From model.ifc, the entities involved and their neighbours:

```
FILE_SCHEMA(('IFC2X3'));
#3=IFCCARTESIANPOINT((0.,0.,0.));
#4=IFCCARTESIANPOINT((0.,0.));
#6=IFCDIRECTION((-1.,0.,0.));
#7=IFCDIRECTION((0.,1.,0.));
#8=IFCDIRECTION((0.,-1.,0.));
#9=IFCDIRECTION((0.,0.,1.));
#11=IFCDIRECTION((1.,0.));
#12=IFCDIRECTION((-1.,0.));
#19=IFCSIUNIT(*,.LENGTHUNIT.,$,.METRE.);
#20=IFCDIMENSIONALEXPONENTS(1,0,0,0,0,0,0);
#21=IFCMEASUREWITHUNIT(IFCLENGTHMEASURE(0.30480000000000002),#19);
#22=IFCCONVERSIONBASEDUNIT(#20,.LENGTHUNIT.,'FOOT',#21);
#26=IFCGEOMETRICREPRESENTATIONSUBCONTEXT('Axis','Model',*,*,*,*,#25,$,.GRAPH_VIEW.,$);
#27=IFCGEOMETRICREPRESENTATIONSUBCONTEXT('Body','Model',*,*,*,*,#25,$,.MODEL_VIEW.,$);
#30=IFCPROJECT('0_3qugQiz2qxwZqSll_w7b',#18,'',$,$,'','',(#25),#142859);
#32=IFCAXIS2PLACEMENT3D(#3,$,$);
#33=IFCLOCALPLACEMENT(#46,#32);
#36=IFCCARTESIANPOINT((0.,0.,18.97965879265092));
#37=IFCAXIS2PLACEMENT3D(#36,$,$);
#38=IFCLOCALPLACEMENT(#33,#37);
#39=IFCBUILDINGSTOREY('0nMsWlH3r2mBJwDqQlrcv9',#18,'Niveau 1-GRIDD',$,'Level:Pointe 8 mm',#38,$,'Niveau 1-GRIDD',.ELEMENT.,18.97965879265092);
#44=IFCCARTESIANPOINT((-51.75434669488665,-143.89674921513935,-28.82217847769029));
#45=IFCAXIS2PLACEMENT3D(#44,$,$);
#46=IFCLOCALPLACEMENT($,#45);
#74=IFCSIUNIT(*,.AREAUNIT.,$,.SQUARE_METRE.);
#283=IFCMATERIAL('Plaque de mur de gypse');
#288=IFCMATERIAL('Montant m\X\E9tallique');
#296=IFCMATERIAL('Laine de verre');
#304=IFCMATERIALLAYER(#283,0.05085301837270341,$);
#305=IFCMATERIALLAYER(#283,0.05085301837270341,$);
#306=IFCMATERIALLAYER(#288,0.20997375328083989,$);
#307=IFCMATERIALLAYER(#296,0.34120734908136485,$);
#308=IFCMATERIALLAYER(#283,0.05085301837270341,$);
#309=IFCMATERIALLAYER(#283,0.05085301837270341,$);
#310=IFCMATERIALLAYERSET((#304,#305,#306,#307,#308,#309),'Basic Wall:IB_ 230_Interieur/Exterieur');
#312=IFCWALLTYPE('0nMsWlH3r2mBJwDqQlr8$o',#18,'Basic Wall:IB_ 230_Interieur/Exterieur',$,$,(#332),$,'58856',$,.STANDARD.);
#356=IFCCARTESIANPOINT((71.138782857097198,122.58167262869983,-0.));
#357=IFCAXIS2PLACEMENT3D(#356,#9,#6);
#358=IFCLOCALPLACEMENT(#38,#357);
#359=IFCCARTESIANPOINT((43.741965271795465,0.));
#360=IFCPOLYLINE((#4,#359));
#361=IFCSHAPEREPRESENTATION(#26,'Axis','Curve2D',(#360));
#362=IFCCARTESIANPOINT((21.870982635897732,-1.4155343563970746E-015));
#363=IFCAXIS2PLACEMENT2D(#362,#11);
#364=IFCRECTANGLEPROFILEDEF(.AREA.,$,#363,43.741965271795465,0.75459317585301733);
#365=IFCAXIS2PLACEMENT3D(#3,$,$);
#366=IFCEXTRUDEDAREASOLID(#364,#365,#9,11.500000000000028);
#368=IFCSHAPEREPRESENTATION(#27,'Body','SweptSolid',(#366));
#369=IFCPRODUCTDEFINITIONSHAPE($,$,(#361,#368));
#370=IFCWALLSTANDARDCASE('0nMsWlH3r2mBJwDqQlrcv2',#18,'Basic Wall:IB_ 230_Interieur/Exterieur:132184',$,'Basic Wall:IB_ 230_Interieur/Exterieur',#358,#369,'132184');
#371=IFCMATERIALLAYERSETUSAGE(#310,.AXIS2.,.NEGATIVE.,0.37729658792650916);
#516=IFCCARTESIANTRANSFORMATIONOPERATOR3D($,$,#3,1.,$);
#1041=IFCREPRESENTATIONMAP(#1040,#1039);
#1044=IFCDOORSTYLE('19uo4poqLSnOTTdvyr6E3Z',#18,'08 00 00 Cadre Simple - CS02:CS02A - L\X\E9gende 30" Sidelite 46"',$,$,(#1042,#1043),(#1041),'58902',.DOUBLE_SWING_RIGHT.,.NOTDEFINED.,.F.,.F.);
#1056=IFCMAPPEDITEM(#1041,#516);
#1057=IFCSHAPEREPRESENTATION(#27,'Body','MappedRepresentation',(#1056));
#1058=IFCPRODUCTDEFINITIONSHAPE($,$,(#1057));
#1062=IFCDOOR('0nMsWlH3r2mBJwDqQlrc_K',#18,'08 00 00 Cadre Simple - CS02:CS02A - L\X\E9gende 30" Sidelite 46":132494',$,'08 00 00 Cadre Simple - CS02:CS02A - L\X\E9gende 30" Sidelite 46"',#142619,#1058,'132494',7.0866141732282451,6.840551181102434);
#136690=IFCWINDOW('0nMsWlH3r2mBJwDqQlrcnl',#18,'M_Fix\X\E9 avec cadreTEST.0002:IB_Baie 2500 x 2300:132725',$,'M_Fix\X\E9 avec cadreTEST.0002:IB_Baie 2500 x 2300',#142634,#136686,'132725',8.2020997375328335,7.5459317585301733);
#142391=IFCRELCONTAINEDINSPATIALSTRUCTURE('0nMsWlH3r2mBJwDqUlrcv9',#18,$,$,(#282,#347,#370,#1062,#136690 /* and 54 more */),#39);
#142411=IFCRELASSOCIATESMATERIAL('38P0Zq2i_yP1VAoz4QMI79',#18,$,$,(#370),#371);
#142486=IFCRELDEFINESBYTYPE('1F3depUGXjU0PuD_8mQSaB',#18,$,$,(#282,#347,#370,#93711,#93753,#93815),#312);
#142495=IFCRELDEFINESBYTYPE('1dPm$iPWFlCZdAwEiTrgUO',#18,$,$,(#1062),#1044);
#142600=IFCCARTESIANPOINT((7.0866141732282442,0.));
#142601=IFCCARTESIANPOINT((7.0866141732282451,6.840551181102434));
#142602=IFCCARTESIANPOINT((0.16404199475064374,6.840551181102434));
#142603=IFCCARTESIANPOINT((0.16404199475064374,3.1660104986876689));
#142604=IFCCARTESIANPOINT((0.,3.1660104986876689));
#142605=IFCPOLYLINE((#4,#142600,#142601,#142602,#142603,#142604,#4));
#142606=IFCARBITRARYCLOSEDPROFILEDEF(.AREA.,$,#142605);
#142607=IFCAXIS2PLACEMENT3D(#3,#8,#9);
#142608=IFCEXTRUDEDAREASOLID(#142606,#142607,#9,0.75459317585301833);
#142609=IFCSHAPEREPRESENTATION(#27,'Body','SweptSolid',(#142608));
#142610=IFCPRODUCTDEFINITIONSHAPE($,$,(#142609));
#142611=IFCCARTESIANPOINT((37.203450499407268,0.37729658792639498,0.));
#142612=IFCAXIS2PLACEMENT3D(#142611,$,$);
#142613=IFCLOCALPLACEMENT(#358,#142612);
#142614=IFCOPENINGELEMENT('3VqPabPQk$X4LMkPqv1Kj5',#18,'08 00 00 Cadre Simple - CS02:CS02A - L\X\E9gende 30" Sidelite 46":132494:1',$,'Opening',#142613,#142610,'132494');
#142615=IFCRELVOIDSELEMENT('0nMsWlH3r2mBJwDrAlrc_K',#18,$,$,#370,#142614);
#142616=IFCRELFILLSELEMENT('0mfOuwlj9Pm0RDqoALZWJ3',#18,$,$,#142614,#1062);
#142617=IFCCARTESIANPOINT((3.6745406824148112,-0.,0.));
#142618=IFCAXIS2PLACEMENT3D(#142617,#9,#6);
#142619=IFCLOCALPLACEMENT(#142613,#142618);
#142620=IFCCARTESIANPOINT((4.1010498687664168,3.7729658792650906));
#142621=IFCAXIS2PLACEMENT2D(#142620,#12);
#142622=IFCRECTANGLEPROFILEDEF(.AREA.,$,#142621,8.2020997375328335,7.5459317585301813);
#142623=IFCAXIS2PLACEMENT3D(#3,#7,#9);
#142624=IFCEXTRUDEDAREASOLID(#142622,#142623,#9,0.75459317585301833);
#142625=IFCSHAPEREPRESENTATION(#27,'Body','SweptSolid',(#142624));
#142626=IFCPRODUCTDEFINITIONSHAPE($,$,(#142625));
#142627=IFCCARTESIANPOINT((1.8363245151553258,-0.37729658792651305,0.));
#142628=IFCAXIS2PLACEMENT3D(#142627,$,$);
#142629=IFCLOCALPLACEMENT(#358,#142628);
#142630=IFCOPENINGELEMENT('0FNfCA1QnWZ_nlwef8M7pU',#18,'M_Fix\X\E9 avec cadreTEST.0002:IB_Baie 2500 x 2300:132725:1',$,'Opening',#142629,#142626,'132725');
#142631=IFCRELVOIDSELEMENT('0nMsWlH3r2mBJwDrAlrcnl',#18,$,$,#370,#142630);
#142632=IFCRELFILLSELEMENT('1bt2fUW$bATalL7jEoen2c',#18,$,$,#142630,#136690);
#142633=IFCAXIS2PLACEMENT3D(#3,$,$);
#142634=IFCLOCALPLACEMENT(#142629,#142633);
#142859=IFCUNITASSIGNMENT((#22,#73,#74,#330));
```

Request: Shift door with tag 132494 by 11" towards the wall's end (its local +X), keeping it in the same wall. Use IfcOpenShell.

```python
import ifcopenshell
import ifcopenshell.api.geometry
import ifcopenshell.util.placement
import ifcopenshell.util.unit

model = ifcopenshell.open("model.ifc")
unit_scale = ifcopenshell.util.unit.calculate_unit_scale(model)

door = model.by_guid("0nMsWlH3r2mBJwDqQlrc_K")
opening = door.FillsVoids[0].RelatingOpeningElement
wall = opening.VoidsElements[0].RelatingBuildingElement

wall_matrix = ifcopenshell.util.placement.get_local_placement(wall.ObjectPlacement)
shift = wall_matrix[:3, 0] * 11 * 0.0254 / unit_scale
before = ifcopenshell.util.placement.get_local_placement(door.ObjectPlacement)[:3, 3].copy()

# The door is placed relative to its opening, so it follows when the opening moves.
matrix = ifcopenshell.util.placement.get_local_placement(opening.ObjectPlacement)
matrix[:3, 3] += shift
ifcopenshell.api.geometry.edit_object_placement(
    model, product=opening, matrix=matrix, is_si=False, should_transform_children=True
)

after = ifcopenshell.util.placement.get_local_placement(door.ObjectPlacement)[:3, 3]
print("door moved by", (after - before).round(3) + 0.0)

model.write("model_rev.ifc")
```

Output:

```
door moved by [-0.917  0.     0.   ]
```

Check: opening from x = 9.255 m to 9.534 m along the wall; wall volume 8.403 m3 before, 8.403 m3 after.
